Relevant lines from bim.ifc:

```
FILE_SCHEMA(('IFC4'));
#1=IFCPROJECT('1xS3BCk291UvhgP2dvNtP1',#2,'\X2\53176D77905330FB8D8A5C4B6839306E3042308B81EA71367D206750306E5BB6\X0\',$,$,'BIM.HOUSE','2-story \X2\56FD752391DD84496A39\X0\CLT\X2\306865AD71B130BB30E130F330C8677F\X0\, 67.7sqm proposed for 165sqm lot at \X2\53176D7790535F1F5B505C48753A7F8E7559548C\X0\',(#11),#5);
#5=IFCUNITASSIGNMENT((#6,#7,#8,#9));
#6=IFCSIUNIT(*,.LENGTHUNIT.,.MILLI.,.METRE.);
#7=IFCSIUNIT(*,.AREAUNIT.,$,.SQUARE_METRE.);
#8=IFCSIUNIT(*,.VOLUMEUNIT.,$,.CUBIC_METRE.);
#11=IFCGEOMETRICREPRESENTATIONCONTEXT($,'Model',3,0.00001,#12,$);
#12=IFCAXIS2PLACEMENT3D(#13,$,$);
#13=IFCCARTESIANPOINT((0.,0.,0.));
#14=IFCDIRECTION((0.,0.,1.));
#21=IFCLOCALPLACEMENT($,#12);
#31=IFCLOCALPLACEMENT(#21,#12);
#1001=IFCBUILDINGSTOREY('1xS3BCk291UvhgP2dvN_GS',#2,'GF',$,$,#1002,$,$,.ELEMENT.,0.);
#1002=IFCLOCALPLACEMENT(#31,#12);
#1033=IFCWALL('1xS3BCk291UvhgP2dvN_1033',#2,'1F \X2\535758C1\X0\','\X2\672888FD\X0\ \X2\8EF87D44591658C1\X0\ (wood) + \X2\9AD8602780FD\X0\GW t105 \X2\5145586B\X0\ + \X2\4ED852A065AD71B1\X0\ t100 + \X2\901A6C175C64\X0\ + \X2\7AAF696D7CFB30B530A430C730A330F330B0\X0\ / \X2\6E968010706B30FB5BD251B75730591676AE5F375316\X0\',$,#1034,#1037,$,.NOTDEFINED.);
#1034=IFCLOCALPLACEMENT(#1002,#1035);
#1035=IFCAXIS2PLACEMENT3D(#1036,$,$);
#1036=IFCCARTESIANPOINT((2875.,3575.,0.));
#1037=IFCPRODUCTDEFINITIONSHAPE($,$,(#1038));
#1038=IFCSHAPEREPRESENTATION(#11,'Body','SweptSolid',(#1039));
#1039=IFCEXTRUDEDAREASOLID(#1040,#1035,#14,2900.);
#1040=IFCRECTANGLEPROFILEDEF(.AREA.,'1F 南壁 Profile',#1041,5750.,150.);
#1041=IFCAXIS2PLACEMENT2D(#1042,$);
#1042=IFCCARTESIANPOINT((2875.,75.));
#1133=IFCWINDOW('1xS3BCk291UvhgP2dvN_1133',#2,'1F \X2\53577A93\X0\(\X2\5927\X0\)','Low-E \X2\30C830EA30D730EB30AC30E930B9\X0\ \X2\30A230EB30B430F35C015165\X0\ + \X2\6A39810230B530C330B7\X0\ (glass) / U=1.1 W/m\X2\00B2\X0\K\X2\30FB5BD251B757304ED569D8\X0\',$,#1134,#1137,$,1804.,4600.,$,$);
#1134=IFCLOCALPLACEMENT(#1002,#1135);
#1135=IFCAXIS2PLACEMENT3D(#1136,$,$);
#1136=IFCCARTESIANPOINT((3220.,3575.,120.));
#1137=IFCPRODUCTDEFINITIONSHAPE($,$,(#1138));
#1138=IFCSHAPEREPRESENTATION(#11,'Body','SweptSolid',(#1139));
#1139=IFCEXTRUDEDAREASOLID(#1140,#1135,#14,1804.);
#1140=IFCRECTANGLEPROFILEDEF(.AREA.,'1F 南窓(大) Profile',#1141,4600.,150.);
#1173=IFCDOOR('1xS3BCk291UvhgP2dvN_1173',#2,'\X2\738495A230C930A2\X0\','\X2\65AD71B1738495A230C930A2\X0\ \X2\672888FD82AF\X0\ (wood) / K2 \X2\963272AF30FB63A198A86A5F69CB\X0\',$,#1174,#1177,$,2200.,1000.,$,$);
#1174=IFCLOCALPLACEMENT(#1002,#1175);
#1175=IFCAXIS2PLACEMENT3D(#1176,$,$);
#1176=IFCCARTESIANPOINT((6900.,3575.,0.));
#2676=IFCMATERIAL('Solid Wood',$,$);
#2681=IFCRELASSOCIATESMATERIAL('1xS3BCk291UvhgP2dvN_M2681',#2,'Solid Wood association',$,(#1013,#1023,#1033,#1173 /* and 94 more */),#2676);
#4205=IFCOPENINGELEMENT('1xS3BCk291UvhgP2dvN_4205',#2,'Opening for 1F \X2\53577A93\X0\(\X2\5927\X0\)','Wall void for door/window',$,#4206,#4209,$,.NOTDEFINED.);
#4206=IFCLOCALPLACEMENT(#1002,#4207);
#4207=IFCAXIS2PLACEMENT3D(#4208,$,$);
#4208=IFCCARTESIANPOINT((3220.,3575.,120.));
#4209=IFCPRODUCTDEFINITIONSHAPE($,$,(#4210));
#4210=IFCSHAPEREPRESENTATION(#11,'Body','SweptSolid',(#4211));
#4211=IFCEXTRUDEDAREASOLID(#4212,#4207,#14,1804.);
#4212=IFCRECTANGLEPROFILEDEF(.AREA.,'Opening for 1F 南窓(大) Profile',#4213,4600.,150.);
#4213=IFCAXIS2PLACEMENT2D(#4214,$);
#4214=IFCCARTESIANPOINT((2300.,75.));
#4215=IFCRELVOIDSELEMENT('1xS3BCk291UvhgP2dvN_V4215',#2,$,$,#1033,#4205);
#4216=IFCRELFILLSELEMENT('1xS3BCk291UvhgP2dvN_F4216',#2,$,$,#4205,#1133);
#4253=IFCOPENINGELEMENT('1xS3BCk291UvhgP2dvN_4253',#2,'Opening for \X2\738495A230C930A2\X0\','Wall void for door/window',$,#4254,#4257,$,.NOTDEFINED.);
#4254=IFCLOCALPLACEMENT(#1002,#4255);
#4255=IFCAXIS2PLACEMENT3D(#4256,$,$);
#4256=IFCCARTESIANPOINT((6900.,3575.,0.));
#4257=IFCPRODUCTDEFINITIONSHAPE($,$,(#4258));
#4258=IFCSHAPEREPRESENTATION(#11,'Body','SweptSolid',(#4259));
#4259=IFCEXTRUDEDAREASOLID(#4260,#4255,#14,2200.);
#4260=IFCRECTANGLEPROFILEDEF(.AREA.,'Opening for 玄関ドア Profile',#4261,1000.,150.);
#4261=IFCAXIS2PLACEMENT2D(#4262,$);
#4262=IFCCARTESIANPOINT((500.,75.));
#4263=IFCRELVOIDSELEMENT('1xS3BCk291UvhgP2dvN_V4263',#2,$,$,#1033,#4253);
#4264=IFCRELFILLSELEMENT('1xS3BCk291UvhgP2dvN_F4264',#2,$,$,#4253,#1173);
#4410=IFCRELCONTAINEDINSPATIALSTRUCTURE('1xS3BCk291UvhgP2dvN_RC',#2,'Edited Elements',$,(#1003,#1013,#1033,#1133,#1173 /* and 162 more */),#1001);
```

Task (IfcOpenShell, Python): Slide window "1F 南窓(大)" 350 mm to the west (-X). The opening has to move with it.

```python
import ifcopenshell
import ifcopenshell.api.geometry
import ifcopenshell.util.placement

model = ifcopenshell.open("bim.ifc")

window = model.by_guid("1xS3BCk291UvhgP2dvN_1133")
opening = window.FillsVoids[0].RelatingOpeningElement
wall = opening.VoidsElements[0].RelatingBuildingElement

wall_matrix = ifcopenshell.util.placement.get_local_placement(wall.ObjectPlacement)
shift = wall_matrix[:3, 0] * -350.0
before = ifcopenshell.util.placement.get_local_placement(window.ObjectPlacement)[:3, 3].copy()

# The window is not placed relative to its opening, so move both.
for product in (opening, window):
    matrix = ifcopenshell.util.placement.get_local_placement(product.ObjectPlacement)
    matrix[:3, 3] += shift
    ifcopenshell.api.geometry.edit_object_placement(model, product=product, matrix=matrix, is_si=False)

after = ifcopenshell.util.placement.get_local_placement(window.ObjectPlacement)[:3, 3]
print("window moved by", (after - before).round(3) + 0.0)

model.write("bim-out.ifc")
```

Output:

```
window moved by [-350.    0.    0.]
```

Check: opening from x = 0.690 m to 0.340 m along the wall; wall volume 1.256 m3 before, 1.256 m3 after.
